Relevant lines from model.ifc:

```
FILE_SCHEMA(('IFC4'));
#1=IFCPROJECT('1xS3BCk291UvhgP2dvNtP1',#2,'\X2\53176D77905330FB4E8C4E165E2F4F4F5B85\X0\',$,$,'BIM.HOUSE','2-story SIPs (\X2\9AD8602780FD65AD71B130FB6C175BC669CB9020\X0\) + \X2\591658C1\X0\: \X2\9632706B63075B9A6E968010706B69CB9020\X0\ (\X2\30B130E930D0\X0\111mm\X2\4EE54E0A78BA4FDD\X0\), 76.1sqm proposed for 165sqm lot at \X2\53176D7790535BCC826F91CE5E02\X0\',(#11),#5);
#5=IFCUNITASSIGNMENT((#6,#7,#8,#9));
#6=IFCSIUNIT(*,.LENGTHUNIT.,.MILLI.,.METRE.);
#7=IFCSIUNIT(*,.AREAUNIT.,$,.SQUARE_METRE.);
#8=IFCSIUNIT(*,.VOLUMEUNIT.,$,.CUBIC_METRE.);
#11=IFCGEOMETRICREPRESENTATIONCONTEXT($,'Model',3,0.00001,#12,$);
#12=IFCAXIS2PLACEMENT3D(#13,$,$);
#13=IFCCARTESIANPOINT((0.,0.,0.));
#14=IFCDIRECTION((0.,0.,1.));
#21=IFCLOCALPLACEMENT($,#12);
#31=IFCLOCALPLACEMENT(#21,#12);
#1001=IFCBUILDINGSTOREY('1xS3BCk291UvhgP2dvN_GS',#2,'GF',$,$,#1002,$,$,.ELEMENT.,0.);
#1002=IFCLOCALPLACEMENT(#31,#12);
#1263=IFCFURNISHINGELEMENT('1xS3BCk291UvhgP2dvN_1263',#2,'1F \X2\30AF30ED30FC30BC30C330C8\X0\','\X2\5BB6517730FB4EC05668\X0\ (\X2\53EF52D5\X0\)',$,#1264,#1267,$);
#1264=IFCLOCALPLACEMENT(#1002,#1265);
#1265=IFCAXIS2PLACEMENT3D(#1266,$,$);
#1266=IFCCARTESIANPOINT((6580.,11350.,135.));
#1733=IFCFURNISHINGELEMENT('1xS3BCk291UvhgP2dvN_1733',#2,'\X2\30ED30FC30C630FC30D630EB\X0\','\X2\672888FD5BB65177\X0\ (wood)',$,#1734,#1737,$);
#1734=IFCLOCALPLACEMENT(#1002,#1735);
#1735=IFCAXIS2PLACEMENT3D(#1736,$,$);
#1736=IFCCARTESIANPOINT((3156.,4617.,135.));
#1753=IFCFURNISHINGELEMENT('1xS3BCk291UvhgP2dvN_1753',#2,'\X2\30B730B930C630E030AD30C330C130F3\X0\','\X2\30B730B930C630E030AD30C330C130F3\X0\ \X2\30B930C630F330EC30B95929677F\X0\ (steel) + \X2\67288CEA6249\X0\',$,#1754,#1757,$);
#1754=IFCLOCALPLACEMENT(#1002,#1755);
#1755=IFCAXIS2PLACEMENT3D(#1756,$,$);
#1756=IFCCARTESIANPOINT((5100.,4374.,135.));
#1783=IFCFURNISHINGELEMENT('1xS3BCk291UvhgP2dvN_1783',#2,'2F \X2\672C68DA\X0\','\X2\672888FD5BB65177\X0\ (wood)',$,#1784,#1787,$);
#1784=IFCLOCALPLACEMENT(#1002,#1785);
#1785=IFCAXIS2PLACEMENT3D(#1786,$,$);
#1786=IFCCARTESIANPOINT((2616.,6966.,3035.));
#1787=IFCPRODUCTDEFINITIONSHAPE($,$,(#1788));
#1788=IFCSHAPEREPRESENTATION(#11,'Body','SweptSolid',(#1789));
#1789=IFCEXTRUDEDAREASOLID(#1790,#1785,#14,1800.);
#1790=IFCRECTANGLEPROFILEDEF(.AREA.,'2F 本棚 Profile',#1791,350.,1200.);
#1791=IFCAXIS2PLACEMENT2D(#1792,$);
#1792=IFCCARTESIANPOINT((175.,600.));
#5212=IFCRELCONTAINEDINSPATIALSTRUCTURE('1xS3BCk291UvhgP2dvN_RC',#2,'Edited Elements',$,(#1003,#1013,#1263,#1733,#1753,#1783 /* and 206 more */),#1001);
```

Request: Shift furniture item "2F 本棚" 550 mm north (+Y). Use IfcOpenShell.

```python
import ifcopenshell
import ifcopenshell.api.geometry
import ifcopenshell.util.placement
import ifcopenshell.util.unit

model = ifcopenshell.open("model.ifc")
unit_scale = ifcopenshell.util.unit.calculate_unit_scale(model)

item = model.by_id(1783)
matrix = ifcopenshell.util.placement.get_local_placement(item.ObjectPlacement)
matrix[1, 3] += 0.55 / unit_scale
ifcopenshell.api.geometry.edit_object_placement(model, product=item, matrix=matrix, is_si=False)

print(ifcopenshell.util.placement.get_local_placement(item.ObjectPlacement).round(3) + 0.0)

model.write("model_edited.ifc")
```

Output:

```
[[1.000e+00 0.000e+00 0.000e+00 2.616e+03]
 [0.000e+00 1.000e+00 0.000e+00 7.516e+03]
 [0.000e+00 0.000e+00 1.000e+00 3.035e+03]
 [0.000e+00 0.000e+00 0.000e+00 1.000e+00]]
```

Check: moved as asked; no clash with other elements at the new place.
